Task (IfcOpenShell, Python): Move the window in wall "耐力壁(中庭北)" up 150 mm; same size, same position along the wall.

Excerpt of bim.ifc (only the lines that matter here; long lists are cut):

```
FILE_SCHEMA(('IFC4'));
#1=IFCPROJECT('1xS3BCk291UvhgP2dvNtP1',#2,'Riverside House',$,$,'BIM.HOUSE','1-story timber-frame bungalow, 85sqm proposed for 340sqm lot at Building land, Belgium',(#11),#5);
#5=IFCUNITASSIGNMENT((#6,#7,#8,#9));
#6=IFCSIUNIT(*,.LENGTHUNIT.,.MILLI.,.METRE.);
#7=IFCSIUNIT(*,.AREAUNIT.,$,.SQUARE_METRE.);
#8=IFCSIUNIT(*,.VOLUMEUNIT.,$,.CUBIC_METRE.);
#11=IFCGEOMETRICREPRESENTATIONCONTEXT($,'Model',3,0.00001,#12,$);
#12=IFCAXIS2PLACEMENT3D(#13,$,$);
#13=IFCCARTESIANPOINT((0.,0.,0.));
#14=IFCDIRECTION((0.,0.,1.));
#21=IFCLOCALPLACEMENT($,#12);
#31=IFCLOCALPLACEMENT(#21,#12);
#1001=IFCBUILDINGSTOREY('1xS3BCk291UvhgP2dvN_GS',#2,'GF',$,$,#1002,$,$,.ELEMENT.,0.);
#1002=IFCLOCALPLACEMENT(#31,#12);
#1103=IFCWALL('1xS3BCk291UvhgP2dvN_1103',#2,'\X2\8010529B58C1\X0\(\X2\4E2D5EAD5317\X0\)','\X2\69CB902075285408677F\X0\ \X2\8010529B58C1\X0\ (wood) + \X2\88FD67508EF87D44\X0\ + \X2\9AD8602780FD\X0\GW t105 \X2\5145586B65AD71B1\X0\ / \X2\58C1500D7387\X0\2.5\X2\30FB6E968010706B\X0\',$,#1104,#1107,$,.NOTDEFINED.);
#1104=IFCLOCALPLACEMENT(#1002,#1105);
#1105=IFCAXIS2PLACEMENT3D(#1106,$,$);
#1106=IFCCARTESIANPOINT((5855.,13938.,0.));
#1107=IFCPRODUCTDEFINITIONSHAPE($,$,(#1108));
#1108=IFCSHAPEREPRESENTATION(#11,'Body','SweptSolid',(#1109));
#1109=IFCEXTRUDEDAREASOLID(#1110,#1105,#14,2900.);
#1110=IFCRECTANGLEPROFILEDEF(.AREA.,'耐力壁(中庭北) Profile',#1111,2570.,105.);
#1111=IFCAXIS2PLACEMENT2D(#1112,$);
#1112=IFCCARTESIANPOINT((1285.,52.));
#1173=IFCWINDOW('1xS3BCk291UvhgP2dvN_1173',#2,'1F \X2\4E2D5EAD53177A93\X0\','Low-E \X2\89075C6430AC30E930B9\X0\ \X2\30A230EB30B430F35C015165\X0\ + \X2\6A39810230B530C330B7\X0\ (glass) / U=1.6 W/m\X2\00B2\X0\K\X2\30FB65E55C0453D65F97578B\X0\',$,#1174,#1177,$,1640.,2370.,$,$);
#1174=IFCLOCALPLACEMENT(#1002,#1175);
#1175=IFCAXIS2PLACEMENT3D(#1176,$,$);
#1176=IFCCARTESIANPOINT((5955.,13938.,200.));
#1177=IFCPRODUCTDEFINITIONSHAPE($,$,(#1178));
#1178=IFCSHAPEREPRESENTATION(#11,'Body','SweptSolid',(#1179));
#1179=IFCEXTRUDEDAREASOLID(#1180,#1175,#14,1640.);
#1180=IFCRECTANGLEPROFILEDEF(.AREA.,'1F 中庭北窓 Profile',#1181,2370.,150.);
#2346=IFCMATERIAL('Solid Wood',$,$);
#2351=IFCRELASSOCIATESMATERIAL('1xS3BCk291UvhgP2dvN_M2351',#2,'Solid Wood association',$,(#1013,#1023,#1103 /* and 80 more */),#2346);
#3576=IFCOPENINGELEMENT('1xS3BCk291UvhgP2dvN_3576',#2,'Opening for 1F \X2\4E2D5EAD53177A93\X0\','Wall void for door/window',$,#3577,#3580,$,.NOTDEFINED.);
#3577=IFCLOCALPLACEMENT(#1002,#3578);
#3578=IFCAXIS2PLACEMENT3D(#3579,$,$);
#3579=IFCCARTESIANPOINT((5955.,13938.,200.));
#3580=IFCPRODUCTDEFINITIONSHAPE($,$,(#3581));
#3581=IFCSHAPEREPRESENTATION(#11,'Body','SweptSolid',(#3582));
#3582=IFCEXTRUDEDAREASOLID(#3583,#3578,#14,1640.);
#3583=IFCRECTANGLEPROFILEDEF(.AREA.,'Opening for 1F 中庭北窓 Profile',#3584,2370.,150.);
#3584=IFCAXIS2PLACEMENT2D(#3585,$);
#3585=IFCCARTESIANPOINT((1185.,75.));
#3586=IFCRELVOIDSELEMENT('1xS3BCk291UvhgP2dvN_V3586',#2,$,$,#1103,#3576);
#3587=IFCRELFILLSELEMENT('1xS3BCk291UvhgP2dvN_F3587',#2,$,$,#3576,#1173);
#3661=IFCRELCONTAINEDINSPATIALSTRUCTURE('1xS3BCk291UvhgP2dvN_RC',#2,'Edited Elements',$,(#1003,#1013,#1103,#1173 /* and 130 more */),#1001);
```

```python
import numpy as np
import ifcopenshell
import ifcopenshell.api.geometry
import ifcopenshell.util.placement
import ifcopenshell.util.unit

model = ifcopenshell.open("bim.ifc")
unit_scale = ifcopenshell.util.unit.calculate_unit_scale(model)

window = model.by_guid("1xS3BCk291UvhgP2dvN_1173")
opening = window.FillsVoids[0].RelatingOpeningElement
dz = 0.15 / unit_scale

shift = np.array([0.0, 0.0, dz])
# The window is not placed relative to its opening, so move both.
for product in (opening, window):
    matrix = ifcopenshell.util.placement.get_local_placement(product.ObjectPlacement)
    matrix[:3, 3] += shift
    ifcopenshell.api.geometry.edit_object_placement(model, product=product, matrix=matrix, is_si=False)

print(f"moved by {dz * unit_scale:+.3f} m")

model.write("bim-out.ifc")
```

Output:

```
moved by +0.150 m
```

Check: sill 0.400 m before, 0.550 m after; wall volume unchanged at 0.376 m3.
